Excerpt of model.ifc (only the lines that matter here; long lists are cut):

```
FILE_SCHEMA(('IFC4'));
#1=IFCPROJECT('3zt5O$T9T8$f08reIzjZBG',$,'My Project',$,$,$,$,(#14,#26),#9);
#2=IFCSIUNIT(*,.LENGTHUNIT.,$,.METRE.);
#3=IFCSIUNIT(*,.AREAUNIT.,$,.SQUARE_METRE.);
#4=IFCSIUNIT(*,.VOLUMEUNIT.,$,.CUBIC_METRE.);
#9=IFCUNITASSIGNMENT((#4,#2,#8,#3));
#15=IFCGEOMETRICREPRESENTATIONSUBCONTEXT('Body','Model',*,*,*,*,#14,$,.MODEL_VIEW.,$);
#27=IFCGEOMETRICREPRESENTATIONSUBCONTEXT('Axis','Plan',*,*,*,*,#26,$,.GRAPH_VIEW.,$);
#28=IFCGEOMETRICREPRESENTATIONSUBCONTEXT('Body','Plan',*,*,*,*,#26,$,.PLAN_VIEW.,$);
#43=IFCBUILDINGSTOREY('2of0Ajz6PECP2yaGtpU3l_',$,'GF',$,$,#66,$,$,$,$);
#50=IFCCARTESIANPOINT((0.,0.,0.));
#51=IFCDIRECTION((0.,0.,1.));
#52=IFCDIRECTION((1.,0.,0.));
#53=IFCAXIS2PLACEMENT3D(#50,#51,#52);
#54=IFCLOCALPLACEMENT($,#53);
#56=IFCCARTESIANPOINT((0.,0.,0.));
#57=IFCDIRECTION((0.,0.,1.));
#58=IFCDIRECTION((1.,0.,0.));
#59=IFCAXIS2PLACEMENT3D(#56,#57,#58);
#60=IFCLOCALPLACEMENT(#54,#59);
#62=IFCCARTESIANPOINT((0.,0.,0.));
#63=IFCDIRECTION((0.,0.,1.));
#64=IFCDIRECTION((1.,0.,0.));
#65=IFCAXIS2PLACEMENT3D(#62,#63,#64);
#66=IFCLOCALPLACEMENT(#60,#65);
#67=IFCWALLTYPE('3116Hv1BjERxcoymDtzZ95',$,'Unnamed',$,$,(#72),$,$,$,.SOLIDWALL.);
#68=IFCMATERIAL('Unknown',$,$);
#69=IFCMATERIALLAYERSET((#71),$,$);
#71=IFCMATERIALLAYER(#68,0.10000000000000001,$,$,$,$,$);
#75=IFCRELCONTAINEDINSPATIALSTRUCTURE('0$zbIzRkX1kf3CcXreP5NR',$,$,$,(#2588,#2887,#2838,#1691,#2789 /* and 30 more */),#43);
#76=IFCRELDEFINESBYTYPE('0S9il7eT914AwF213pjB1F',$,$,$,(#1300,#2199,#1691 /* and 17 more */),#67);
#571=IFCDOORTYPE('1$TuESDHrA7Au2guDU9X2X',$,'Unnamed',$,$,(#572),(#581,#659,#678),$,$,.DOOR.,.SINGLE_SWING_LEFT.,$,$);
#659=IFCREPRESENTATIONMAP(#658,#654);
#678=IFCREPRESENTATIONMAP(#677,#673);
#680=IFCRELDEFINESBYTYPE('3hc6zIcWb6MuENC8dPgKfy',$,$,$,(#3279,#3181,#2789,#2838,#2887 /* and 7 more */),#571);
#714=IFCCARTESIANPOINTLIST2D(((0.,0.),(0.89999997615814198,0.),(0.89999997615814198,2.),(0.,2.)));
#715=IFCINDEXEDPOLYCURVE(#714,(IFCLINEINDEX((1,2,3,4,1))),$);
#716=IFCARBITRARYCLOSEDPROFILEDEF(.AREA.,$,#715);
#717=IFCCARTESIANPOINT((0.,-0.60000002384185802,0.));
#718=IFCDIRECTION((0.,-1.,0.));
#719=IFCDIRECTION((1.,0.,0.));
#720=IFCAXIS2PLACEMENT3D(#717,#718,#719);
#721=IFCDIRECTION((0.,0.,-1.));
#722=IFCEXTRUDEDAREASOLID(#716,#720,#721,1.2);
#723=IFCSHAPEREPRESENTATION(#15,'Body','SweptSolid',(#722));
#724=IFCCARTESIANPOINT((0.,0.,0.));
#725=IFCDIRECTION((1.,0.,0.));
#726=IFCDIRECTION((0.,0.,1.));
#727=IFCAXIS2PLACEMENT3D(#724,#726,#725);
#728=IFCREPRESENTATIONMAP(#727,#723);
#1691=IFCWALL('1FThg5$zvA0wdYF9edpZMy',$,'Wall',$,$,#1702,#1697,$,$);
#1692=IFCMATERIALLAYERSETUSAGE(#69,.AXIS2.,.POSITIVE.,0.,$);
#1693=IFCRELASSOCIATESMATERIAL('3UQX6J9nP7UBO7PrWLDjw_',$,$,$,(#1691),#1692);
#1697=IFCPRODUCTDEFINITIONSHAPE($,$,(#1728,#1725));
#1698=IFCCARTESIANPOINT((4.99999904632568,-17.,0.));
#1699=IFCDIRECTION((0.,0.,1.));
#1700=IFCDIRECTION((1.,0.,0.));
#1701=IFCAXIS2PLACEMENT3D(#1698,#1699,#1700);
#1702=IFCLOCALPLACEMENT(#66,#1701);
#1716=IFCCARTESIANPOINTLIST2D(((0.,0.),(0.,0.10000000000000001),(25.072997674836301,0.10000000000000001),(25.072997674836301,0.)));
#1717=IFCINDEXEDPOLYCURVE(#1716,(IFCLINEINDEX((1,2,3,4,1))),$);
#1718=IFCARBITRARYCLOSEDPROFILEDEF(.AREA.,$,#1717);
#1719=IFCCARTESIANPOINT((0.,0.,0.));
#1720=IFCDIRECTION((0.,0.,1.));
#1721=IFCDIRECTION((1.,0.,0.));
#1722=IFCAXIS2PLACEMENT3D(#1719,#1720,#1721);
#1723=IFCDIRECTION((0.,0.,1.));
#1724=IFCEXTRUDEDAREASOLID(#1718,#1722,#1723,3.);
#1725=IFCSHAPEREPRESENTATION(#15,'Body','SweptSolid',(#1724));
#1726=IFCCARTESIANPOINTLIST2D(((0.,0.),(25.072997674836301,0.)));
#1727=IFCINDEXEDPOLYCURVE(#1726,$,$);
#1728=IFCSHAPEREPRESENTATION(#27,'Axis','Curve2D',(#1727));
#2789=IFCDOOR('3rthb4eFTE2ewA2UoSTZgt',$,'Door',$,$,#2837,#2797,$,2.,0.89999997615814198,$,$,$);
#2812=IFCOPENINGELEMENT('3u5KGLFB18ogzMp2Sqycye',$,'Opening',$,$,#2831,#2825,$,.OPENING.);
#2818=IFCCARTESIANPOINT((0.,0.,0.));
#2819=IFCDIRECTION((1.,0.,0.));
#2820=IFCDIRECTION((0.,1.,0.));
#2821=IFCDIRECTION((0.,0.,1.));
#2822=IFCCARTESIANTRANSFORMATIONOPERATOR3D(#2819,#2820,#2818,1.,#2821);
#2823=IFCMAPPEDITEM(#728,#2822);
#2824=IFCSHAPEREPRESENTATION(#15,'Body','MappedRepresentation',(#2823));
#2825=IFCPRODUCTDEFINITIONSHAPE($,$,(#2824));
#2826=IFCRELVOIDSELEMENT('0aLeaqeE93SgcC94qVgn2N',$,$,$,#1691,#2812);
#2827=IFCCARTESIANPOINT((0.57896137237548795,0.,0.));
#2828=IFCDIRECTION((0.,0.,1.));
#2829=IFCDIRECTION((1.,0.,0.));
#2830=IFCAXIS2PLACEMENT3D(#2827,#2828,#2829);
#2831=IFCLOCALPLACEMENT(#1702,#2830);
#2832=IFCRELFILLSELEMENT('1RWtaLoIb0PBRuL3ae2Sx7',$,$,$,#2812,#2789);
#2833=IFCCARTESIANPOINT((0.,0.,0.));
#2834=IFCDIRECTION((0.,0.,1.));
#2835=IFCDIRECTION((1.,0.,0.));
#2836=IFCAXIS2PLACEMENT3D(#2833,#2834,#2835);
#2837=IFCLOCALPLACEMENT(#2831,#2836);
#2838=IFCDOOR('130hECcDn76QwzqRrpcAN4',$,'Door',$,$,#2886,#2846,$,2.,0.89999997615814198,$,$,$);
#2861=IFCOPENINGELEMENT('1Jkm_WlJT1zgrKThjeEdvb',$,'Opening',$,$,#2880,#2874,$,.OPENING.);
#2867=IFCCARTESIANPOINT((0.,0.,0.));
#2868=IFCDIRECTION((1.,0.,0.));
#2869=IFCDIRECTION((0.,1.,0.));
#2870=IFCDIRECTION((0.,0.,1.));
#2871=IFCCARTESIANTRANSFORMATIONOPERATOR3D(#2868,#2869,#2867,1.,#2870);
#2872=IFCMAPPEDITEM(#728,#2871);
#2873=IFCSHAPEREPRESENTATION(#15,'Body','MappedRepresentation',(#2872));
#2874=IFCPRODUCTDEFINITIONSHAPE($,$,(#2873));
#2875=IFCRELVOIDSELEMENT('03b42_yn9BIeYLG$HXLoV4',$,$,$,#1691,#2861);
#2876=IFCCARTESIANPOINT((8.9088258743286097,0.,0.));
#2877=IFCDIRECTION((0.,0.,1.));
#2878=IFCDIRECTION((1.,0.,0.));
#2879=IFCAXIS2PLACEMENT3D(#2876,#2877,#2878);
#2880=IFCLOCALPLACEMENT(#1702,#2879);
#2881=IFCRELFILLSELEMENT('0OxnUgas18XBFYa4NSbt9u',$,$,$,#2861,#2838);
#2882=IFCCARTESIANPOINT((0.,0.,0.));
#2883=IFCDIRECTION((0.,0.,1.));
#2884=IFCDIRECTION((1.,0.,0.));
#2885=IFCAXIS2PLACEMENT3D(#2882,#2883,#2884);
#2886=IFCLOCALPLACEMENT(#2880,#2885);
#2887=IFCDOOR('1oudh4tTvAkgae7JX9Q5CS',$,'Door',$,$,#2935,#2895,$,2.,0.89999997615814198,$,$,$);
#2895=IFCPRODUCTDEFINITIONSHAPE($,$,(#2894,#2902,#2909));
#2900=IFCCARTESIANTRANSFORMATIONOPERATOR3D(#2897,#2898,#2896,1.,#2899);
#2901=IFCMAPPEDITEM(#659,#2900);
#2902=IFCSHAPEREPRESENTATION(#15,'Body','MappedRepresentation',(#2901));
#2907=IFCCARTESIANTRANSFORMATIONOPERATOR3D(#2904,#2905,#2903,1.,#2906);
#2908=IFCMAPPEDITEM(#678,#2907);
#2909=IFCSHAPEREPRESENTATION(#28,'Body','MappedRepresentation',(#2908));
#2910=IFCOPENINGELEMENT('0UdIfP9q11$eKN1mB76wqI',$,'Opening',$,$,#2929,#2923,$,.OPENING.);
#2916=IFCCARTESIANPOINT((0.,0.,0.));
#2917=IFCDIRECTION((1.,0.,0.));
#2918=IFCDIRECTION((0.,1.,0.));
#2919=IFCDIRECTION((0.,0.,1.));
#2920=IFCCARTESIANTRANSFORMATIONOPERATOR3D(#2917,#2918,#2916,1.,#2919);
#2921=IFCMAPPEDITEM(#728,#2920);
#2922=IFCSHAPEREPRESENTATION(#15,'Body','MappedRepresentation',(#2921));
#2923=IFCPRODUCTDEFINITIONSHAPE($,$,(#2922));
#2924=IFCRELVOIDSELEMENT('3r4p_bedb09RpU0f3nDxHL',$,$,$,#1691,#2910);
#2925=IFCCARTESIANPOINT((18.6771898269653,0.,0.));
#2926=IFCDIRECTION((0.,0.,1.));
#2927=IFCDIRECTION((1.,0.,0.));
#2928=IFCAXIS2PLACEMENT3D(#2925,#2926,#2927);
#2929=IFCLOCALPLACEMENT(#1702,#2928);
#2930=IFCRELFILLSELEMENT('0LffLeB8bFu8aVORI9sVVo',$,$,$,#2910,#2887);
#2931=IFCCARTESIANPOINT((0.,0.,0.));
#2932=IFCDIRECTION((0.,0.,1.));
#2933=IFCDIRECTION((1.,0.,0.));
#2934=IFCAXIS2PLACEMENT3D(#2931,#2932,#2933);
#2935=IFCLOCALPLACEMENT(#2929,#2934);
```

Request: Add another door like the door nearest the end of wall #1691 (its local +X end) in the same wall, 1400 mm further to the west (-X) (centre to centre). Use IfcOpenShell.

```python
import ifcopenshell
import ifcopenshell.api.feature
import ifcopenshell.api.geometry
import ifcopenshell.api.root
import ifcopenshell.geom
import ifcopenshell.util.element
import ifcopenshell.util.placement
import ifcopenshell.util.shape

model = ifcopenshell.open("model.ifc")
settings = ifcopenshell.geom.settings()


def volume(element):
    """Net volume in cubic metres, openings subtracted."""
    shape = ifcopenshell.geom.create_shape(settings, element)
    return ifcopenshell.util.shape.get_volume(shape.geometry)


door = model.by_guid("1oudh4tTvAkgae7JX9Q5CS")
opening = door.FillsVoids[0].RelatingOpeningElement
wall = opening.VoidsElements[0].RelatingBuildingElement
before = volume(wall)
shift = ifcopenshell.util.placement.get_local_placement(wall.ObjectPlacement)[:3, 0] * -1.4

# copy_class copies the void relationship, type, container and properties, but no geometry.
new_opening = ifcopenshell.api.root.copy_class(model, product=opening)
new_opening.Representation = ifcopenshell.util.element.copy_deep(
    model, opening.Representation, exclude=["IfcGeometricRepresentationContext", "IfcRepresentationMap"]
)
new_door = ifcopenshell.api.root.copy_class(model, product=door)
new_door.Representation = ifcopenshell.util.element.copy_deep(
    model, door.Representation, exclude=["IfcGeometricRepresentationContext", "IfcRepresentationMap"]
)
ifcopenshell.api.feature.add_filling(model, opening=new_opening, element=new_door)

for old, new in ((opening, new_opening), (door, new_door)):
    matrix = ifcopenshell.util.placement.get_local_placement(old.ObjectPlacement)
    matrix[:3, 3] += shift
    ifcopenshell.api.geometry.edit_object_placement(model, product=new, matrix=matrix, is_si=False)

after = volume(wall)

print(f"wall volume {before:.3f} -> {after:.3f} m3")

model.write("model_v2.ifc")
```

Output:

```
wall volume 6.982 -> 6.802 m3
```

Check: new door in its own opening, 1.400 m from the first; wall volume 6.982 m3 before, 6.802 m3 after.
